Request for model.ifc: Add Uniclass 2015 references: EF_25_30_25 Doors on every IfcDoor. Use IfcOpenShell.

First a look at what the model holds.

```python
import ifcopenshell

model = ifcopenshell.open("model.ifc")
print(model.schema)
print("classifications:", [c.Name for c in model.by_type("IfcClassification")])
for ifc_class in ("IfcDoor", "IfcRoof", "IfcStair", "IfcWall", "IfcWindow"):
    print(ifc_class, len(model.by_type(ifc_class)))
```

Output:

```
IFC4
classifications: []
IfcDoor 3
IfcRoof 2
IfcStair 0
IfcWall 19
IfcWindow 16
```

```python
import ifcopenshell
import ifcopenshell.api.classification

model = ifcopenshell.open("model.ifc")

system = ifcopenshell.api.classification.add_classification(model, classification="Uniclass 2015")

codes = {
    "IfcDoor": ("EF_25_30_25", "Doors"),
}
for ifc_class, (code, name) in codes.items():
    products = model.by_type(ifc_class)
    ifcopenshell.api.classification.add_reference(
        model, products=products, classification=system, identification=code, name=name
    )
    print(code, len(products))

model.write("model_edited.ifc")
```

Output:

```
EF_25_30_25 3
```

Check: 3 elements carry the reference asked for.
